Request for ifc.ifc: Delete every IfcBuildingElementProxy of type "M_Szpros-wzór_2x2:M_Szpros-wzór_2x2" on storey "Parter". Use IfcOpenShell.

First a look at what the model holds.

```python
import ifcopenshell
import ifcopenshell.util.element

model = ifcopenshell.open("ifc.ifc")
print(model.schema)
storey = next(s for s in model.by_type("IfcBuildingStorey") if s.Name == "Parter")
proxies = [e for e in ifcopenshell.util.element.get_decomposition(storey) if e.is_a("IfcBuildingElementProxy")]
seen = {}
for e in proxies:
    element_type = ifcopenshell.util.element.get_type(e)
    name = element_type.Name if element_type not in (None, e) else None
    seen[name] = seen.get(name, 0) + 1
for name, count in sorted(seen.items(), key=str):
    print(count, "x", name)
```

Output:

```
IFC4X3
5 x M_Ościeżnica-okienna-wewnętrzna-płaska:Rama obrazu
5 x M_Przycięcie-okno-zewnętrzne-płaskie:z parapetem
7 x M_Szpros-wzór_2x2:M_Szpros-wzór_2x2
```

```python
import ifcopenshell
import ifcopenshell.api.root
import ifcopenshell.util.element

model = ifcopenshell.open("ifc.ifc")

storey = next(s for s in model.by_type("IfcBuildingStorey") if s.Name == "Parter")
proxies = [e for e in ifcopenshell.util.element.get_decomposition(storey) if e.is_a("IfcBuildingElementProxy")]
targets = [e for e in proxies if (t := ifcopenshell.util.element.get_type(e)) not in (None, e) and t.Name == "M_Szpros-wzór_2x2:M_Szpros-wzór_2x2"]

for e in targets:
    ifcopenshell.api.root.remove_product(model, product=e)
print(len(targets), "removed")

model.write("ifc_v2.ifc")
```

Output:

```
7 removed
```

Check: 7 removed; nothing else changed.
